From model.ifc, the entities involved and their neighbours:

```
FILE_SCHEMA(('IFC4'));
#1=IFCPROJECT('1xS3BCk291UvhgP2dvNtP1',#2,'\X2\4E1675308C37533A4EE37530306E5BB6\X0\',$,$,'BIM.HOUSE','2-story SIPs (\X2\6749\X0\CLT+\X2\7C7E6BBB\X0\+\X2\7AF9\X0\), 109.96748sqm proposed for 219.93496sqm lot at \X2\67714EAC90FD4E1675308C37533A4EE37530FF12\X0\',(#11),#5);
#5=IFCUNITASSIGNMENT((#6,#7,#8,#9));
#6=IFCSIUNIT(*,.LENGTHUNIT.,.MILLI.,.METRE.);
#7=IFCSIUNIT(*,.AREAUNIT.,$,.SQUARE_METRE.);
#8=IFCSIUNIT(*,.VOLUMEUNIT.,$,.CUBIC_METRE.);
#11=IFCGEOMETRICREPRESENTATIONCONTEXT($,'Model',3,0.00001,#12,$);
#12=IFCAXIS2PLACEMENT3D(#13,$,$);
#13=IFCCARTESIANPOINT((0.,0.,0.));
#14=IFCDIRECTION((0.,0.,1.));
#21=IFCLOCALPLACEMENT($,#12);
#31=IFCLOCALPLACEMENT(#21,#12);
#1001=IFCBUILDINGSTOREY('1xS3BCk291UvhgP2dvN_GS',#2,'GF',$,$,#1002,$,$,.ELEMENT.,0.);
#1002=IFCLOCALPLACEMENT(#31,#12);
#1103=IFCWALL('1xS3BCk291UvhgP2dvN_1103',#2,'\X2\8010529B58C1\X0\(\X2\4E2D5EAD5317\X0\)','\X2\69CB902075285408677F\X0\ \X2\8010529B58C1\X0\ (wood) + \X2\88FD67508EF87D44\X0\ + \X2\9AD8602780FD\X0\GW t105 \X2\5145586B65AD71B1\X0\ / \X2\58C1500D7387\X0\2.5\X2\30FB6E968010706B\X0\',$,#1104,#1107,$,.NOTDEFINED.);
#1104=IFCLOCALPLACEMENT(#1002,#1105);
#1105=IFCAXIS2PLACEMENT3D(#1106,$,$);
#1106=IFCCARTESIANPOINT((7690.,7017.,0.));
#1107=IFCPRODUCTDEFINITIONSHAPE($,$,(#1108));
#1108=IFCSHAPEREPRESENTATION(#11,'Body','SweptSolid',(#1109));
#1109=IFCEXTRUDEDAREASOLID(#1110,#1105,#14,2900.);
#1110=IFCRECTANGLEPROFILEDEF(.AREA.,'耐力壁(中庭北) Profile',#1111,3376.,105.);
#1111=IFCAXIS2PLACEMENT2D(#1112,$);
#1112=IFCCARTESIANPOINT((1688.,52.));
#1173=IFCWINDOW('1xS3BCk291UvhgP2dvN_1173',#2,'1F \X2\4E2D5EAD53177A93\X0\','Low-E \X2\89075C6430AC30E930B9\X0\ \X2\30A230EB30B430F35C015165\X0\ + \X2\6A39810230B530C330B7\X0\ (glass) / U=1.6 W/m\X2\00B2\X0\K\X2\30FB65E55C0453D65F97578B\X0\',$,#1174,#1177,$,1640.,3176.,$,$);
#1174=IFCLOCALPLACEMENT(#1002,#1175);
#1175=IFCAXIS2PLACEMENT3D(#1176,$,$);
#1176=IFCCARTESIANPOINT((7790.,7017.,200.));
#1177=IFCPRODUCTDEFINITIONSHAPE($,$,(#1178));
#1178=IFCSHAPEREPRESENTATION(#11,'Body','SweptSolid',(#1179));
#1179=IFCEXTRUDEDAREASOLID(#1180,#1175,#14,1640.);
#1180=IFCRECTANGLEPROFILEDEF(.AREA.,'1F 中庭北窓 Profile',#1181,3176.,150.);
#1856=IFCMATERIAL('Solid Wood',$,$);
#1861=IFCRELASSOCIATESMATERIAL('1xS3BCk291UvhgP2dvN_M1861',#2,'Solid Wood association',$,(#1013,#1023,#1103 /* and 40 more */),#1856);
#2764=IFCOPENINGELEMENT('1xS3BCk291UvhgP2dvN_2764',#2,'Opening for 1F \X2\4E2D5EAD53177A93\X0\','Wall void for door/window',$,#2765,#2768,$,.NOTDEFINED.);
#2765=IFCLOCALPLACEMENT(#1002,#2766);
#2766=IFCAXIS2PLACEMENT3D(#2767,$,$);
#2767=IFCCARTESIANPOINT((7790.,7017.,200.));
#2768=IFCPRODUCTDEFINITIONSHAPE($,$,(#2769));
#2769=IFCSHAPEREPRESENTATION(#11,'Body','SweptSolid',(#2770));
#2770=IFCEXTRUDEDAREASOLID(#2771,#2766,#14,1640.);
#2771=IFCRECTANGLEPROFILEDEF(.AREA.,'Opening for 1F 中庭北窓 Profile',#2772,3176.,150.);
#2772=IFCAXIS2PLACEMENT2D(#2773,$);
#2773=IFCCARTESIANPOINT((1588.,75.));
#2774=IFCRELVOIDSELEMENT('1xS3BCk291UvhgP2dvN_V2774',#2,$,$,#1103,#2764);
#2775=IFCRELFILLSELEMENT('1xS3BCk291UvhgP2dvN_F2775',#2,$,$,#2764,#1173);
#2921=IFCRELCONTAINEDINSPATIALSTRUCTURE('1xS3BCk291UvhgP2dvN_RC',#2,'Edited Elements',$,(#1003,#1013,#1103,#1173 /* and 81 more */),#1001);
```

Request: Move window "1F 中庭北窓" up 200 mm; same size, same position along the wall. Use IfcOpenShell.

```python
import numpy as np
import ifcopenshell
import ifcopenshell.api.geometry
import ifcopenshell.util.placement
import ifcopenshell.util.unit

model = ifcopenshell.open("model.ifc")
unit_scale = ifcopenshell.util.unit.calculate_unit_scale(model)

window = model.by_guid("1xS3BCk291UvhgP2dvN_1173")
opening = window.FillsVoids[0].RelatingOpeningElement
dz = 0.2 / unit_scale

shift = np.array([0.0, 0.0, dz])
# The window is not placed relative to its opening, so move both.
for product in (opening, window):
    matrix = ifcopenshell.util.placement.get_local_placement(product.ObjectPlacement)
    matrix[:3, 3] += shift
    ifcopenshell.api.geometry.edit_object_placement(model, product=product, matrix=matrix, is_si=False)

print(f"moved by {dz * unit_scale:+.3f} m")

model.write("model_rev.ifc")
```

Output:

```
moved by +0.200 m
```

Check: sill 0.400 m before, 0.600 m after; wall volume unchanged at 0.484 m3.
